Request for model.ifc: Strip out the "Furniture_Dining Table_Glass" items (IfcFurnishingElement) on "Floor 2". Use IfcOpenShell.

First a look at what the model holds.

```python
import ifcopenshell
import ifcopenshell.util.element

model = ifcopenshell.open("model.ifc")
print(model.schema)
storey = next(s for s in model.by_type("IfcBuildingStorey") if s.Name == "Floor 2")
furniture = [e for e in ifcopenshell.util.element.get_decomposition(storey) if e.is_a("IfcFurnishingElement")]
seen = {}
for e in furniture:
    element_type = ifcopenshell.util.element.get_type(e)
    name = element_type.Name if element_type not in (None, e) else None
    seen[name] = seen.get(name, 0) + 1
for name, count in sorted(seen.items(), key=str):
    print(count, "x", name)
```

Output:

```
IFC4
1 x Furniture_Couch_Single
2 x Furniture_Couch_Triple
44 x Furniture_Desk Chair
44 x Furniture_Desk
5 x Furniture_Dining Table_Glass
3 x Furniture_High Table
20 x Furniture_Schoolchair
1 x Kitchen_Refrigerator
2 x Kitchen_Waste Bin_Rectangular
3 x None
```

```python
import ifcopenshell
import ifcopenshell.api.root
import ifcopenshell.util.element

model = ifcopenshell.open("model.ifc")

storey = next(s for s in model.by_type("IfcBuildingStorey") if s.Name == "Floor 2")
furniture = [e for e in ifcopenshell.util.element.get_decomposition(storey) if e.is_a("IfcFurnishingElement")]
targets = [e for e in furniture if (t := ifcopenshell.util.element.get_type(e)) not in (None, e) and t.Name == "Furniture_Dining Table_Glass"]

for e in targets:
    ifcopenshell.api.root.remove_product(model, product=e)
print(len(targets), "removed")

model.write("model_v2.ifc")
```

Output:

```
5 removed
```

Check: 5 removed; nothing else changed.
